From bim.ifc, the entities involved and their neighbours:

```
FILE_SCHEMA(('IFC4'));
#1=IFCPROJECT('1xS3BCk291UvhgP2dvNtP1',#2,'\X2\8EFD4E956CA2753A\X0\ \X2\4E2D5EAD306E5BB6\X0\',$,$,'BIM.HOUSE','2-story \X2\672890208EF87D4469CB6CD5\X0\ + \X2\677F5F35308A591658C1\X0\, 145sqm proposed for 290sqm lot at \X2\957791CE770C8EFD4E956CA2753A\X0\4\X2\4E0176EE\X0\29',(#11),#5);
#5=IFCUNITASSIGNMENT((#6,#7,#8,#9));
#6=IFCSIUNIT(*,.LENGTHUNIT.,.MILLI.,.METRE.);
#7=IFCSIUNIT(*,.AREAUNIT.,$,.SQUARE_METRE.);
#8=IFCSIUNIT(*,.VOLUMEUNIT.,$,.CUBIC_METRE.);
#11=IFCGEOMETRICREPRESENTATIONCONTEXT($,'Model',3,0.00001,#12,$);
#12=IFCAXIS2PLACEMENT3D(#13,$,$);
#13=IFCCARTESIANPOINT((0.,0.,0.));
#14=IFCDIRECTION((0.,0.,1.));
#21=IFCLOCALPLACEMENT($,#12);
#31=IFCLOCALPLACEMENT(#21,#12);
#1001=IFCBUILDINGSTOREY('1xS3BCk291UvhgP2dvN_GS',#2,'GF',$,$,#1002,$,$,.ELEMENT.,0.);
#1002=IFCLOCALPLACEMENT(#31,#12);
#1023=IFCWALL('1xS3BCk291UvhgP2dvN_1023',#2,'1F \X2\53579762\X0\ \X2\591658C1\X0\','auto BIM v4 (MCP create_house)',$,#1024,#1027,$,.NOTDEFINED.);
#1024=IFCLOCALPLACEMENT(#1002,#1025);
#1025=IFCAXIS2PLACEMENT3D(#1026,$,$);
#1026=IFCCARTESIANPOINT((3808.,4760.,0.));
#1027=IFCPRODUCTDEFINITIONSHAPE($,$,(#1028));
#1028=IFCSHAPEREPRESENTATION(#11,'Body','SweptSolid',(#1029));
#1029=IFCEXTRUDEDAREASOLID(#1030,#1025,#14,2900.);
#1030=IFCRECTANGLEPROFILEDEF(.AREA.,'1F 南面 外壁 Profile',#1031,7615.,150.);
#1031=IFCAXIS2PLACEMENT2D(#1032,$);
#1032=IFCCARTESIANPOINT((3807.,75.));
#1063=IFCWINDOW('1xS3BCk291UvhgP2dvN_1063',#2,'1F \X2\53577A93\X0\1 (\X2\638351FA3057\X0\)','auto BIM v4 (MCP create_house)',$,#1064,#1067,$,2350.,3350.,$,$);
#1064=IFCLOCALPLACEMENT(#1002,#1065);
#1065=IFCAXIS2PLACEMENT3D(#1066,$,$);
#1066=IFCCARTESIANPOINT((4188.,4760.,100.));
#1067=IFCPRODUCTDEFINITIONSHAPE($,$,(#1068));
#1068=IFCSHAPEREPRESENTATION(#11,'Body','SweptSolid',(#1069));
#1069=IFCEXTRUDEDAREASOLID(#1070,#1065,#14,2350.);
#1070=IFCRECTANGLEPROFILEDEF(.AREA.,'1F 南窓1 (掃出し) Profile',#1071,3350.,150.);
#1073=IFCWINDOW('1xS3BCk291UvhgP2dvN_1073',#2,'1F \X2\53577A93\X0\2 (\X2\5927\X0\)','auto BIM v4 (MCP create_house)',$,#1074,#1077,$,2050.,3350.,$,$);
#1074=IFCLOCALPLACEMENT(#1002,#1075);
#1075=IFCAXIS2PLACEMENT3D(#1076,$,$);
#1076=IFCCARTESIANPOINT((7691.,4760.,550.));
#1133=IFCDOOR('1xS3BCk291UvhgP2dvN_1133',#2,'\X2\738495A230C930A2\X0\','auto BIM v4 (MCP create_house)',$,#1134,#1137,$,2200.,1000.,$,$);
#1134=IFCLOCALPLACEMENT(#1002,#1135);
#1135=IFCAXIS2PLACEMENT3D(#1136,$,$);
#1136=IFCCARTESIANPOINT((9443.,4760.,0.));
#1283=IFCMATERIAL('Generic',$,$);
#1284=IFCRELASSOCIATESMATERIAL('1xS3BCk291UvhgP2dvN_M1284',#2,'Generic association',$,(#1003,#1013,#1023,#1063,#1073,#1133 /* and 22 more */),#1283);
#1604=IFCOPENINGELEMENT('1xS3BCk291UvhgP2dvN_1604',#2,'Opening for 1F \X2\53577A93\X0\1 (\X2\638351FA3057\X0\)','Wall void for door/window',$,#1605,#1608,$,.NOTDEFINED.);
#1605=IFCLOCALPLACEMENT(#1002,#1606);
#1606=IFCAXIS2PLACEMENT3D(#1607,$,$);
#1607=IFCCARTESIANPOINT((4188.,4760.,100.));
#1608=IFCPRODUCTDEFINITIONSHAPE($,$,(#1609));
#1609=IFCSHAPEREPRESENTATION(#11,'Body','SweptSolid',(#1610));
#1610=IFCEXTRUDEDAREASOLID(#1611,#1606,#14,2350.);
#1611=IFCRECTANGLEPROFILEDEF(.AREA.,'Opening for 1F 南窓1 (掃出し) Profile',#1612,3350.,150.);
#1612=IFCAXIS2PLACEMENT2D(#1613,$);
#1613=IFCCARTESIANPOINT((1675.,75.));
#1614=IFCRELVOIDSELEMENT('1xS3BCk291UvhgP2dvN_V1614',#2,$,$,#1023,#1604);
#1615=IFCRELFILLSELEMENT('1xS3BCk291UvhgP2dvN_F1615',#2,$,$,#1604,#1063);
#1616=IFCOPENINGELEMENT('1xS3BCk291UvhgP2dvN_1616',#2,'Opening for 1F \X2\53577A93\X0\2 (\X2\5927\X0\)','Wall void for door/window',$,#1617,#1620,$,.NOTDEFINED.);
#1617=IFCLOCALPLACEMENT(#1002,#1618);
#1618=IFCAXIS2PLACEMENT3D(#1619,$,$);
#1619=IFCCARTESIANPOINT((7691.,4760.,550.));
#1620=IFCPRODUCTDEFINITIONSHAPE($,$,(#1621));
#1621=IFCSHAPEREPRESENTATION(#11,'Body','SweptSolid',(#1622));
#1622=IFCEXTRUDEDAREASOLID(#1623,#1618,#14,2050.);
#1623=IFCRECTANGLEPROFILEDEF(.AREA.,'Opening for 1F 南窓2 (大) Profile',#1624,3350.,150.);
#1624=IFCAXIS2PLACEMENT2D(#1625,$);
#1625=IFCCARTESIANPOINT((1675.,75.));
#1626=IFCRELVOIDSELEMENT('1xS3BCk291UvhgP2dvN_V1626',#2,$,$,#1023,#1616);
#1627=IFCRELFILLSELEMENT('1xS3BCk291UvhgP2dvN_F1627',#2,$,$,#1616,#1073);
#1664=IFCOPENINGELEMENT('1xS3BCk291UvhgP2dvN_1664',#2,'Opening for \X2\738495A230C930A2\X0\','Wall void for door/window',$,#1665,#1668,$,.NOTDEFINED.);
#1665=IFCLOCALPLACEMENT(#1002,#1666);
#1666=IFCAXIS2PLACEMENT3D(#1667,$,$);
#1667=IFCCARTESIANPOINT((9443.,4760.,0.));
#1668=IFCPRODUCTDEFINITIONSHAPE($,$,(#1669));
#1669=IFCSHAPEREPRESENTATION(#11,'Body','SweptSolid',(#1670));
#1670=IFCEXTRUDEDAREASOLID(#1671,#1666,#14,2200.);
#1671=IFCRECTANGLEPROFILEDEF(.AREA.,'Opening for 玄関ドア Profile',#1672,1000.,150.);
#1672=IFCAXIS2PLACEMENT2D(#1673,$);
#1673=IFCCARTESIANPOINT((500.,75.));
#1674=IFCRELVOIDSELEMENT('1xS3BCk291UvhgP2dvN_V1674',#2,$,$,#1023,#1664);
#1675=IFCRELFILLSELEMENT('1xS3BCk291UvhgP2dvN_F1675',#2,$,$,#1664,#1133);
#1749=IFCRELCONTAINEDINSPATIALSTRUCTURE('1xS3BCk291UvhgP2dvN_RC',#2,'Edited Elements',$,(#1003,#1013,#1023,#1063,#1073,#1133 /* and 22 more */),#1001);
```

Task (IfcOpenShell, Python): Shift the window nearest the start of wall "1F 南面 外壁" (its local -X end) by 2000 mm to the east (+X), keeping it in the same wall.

```python
import ifcopenshell
import ifcopenshell.api.geometry
import ifcopenshell.util.placement

model = ifcopenshell.open("bim.ifc")

window = model.by_guid("1xS3BCk291UvhgP2dvN_1063")
opening = window.FillsVoids[0].RelatingOpeningElement
wall = opening.VoidsElements[0].RelatingBuildingElement

wall_matrix = ifcopenshell.util.placement.get_local_placement(wall.ObjectPlacement)
shift = wall_matrix[:3, 0] * 2000.0
before = ifcopenshell.util.placement.get_local_placement(window.ObjectPlacement)[:3, 3].copy()

# The window is not placed relative to its opening, so move both.
for product in (opening, window):
    matrix = ifcopenshell.util.placement.get_local_placement(product.ObjectPlacement)
    matrix[:3, 3] += shift
    ifcopenshell.api.geometry.edit_object_placement(model, product=product, matrix=matrix, is_si=False)

after = ifcopenshell.util.placement.get_local_placement(window.ObjectPlacement)[:3, 3]
print("window moved by", (after - before).round(3) + 0.0)

model.write("bim_edited.ifc")
```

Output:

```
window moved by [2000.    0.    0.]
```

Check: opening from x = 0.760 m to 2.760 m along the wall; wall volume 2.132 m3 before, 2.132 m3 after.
